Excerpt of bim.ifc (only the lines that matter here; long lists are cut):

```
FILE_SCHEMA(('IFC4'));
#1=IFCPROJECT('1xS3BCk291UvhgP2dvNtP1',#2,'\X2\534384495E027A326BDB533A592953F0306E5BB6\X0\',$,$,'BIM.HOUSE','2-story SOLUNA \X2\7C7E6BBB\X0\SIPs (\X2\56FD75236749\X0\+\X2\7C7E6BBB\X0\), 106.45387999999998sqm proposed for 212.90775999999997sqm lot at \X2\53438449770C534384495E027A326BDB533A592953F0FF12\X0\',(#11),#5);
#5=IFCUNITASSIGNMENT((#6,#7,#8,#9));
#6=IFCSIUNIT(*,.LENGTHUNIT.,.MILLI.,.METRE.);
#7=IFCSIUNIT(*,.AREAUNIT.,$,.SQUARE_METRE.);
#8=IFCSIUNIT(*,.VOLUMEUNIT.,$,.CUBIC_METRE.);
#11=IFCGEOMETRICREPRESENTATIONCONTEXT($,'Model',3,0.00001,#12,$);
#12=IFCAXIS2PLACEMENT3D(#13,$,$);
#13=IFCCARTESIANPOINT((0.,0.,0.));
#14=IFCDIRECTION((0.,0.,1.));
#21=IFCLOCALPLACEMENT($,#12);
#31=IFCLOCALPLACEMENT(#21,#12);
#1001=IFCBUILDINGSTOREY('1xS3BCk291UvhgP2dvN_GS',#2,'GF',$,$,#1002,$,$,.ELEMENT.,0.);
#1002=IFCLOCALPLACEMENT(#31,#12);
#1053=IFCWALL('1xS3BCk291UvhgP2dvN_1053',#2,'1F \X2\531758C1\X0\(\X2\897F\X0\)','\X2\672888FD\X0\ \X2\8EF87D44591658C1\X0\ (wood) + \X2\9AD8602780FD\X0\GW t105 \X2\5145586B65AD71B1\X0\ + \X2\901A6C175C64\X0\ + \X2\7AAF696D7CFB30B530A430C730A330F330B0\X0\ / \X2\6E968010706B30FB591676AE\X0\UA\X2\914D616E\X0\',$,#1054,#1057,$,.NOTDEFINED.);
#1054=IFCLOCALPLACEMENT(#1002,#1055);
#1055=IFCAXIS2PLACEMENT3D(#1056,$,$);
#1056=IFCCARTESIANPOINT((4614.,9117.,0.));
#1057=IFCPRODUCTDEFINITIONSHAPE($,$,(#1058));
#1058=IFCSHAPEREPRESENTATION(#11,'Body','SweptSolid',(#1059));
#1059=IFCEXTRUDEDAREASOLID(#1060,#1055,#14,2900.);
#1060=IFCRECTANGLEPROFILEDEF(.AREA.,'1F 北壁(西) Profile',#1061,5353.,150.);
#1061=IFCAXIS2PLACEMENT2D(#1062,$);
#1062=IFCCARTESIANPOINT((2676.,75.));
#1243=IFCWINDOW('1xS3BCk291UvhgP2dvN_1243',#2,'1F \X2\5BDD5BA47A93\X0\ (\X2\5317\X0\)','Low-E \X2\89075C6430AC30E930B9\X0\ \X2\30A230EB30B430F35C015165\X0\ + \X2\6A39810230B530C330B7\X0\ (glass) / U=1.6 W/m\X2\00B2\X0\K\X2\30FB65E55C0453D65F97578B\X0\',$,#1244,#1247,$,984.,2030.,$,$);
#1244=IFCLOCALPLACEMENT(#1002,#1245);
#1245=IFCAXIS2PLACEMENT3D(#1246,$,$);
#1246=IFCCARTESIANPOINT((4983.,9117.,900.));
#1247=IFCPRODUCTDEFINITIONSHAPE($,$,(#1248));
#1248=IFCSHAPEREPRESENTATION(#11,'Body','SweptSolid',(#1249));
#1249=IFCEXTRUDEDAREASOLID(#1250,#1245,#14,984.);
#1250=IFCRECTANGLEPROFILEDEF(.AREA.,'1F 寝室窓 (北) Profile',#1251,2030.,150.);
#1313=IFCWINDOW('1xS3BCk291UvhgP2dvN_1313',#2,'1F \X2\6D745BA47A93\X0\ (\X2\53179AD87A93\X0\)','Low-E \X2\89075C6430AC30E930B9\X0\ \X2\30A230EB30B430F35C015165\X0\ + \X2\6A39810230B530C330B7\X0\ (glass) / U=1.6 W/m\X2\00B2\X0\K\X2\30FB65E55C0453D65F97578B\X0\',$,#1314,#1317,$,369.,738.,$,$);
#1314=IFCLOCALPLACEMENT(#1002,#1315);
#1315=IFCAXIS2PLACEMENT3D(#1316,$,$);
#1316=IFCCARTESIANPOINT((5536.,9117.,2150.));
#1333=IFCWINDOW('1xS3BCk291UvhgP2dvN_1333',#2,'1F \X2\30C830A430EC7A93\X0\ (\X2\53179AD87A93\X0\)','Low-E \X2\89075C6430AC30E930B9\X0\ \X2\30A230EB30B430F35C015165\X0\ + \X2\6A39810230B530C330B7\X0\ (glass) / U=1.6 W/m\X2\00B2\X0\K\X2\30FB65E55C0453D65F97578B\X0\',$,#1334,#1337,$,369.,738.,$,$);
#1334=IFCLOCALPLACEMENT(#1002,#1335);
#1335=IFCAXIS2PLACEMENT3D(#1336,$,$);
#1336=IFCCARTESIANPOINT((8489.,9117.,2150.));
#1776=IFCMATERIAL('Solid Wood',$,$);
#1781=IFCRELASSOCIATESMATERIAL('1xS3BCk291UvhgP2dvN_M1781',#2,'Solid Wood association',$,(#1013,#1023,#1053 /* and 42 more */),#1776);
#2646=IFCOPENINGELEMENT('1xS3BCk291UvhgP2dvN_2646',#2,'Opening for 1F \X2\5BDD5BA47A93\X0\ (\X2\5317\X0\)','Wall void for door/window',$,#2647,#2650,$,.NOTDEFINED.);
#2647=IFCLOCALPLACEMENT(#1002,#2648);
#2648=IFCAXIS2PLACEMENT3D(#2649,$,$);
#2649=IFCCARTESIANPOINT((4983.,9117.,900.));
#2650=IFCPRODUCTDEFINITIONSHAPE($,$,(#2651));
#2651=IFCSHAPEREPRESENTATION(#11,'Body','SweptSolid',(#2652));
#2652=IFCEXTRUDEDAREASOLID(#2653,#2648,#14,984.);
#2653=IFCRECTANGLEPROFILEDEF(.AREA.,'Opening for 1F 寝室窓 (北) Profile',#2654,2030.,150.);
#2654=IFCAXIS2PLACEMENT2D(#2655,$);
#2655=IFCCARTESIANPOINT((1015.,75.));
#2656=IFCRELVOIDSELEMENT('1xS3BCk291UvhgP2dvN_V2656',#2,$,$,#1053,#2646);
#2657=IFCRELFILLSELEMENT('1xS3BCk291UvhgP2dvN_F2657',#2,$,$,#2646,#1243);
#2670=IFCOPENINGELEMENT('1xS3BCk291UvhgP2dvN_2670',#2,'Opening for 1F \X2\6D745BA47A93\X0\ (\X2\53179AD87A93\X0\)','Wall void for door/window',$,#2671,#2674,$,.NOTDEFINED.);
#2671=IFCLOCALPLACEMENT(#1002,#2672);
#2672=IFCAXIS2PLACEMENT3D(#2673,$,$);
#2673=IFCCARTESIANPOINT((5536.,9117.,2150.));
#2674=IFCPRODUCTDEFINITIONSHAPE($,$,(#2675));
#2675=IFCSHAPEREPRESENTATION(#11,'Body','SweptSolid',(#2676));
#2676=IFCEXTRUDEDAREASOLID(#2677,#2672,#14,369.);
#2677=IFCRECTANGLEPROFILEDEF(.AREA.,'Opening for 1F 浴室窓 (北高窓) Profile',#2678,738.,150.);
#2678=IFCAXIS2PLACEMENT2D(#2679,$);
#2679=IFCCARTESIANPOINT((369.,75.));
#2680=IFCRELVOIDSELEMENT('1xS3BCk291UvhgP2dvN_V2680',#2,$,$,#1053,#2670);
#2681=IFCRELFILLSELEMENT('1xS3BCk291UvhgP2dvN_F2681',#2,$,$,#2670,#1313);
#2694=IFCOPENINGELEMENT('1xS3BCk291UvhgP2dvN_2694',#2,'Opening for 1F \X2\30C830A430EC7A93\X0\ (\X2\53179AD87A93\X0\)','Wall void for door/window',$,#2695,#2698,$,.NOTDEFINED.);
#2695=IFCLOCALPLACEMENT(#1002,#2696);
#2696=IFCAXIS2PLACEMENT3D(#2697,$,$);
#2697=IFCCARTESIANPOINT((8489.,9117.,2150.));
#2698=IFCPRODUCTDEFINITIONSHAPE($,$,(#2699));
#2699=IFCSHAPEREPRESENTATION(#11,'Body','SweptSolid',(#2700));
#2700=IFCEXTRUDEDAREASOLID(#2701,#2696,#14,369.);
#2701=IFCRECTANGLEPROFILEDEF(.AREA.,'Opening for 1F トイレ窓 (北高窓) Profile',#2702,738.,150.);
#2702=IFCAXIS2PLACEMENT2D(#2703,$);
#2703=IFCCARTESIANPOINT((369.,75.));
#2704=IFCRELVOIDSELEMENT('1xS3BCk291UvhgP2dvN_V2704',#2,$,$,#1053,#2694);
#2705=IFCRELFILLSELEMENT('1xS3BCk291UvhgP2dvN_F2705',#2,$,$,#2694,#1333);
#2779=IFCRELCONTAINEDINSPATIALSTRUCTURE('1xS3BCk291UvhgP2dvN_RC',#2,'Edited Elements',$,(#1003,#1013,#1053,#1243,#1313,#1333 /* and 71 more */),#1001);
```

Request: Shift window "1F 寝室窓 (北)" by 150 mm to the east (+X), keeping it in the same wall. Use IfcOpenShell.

```python
import ifcopenshell
import ifcopenshell.api.geometry
import ifcopenshell.util.placement
import ifcopenshell.util.unit

model = ifcopenshell.open("bim.ifc")
unit_scale = ifcopenshell.util.unit.calculate_unit_scale(model)

window = model.by_guid("1xS3BCk291UvhgP2dvN_1243")
opening = window.FillsVoids[0].RelatingOpeningElement
wall = opening.VoidsElements[0].RelatingBuildingElement

wall_matrix = ifcopenshell.util.placement.get_local_placement(wall.ObjectPlacement)
shift = wall_matrix[:3, 0] * 0.15 / unit_scale
before = ifcopenshell.util.placement.get_local_placement(window.ObjectPlacement)[:3, 3].copy()

# The window is not placed relative to its opening, so move both.
for product in (opening, window):
    matrix = ifcopenshell.util.placement.get_local_placement(product.ObjectPlacement)
    matrix[:3, 3] += shift
    ifcopenshell.api.geometry.edit_object_placement(model, product=product, matrix=matrix, is_si=False)

after = ifcopenshell.util.placement.get_local_placement(window.ObjectPlacement)[:3, 3]
print("window moved by", (after - before).round(3) + 0.0)

model.write("bim_edited.ifc")
```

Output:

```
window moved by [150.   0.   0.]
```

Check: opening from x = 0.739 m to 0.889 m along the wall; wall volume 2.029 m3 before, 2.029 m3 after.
